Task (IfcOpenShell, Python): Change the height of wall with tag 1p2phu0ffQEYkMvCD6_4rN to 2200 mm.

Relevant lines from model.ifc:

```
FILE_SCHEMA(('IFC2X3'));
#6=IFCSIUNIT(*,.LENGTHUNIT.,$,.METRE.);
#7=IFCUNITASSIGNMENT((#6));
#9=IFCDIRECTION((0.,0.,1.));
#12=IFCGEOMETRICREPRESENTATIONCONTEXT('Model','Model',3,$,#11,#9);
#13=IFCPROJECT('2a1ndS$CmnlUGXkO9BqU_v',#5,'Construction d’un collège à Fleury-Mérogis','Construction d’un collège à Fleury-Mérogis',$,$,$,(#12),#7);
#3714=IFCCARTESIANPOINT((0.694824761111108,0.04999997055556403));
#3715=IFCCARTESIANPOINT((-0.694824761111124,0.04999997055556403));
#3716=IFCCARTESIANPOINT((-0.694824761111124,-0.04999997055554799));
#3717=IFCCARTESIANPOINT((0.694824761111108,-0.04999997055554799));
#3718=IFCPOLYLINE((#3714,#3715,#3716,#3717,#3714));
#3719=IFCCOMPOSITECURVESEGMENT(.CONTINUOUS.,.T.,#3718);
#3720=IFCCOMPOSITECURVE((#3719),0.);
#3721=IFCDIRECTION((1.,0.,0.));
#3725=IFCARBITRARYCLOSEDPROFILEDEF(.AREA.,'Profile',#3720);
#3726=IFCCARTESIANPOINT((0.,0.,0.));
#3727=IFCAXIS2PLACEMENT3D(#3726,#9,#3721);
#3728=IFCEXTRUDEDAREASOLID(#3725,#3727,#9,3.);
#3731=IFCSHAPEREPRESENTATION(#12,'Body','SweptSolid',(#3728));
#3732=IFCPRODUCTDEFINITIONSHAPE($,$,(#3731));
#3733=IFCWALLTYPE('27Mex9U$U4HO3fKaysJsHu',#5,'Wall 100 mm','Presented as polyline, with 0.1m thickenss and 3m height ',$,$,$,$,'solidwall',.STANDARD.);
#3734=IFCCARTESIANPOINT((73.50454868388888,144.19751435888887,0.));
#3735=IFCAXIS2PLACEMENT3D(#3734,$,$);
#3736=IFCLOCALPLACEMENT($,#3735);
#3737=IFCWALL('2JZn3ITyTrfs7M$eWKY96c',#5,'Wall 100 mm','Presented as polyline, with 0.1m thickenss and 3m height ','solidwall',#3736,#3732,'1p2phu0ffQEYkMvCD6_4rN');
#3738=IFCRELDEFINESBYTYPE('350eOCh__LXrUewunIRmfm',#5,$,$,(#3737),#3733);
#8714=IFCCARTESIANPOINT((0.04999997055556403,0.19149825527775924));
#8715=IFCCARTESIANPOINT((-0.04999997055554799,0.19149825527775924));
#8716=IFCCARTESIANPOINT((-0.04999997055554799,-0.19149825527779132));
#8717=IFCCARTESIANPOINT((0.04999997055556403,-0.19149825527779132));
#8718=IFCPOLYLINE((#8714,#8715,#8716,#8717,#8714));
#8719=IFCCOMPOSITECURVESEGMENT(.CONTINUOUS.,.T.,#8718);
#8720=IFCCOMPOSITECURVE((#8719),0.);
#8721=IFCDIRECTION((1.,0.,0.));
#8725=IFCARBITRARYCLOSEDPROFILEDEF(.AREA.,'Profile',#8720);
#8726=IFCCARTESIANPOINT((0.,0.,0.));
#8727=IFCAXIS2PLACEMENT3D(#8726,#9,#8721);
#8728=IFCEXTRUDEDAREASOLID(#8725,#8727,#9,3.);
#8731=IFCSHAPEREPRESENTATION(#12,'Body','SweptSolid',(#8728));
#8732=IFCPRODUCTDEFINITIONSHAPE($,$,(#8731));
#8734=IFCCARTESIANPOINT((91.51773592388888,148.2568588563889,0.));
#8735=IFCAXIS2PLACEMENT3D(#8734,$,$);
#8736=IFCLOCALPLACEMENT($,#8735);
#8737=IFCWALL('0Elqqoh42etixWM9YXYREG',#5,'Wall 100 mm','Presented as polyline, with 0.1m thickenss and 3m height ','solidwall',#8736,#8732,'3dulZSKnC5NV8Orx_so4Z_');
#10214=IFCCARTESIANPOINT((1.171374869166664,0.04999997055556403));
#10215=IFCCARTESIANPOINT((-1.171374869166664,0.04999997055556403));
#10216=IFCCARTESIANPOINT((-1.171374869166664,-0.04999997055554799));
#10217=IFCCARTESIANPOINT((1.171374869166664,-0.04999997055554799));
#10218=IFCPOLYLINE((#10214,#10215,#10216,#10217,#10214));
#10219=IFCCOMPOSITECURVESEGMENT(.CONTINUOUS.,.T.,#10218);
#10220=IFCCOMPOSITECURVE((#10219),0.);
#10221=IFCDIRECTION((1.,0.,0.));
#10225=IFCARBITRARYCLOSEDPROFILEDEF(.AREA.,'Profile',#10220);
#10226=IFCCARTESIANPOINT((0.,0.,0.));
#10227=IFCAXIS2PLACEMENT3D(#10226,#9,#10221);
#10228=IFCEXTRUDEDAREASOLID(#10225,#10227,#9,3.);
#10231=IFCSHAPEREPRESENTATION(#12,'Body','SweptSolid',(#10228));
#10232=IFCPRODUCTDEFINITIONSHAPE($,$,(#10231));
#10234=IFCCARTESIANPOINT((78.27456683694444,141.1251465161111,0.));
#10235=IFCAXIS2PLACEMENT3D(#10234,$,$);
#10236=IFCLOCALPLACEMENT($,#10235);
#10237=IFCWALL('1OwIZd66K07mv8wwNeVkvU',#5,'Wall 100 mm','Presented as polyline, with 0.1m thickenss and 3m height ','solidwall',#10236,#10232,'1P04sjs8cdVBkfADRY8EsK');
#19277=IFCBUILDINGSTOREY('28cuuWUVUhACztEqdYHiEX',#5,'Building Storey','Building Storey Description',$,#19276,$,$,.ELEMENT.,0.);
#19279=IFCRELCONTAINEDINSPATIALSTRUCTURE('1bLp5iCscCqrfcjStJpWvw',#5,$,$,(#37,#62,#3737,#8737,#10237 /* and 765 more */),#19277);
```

```python
import ifcopenshell
import ifcopenshell.geom
import ifcopenshell.util.shape

model = ifcopenshell.open("model.ifc")
settings = ifcopenshell.geom.settings()


def volume(element):
    """Net volume in cubic metres, openings subtracted."""
    shape = ifcopenshell.geom.create_shape(settings, element)
    return ifcopenshell.util.shape.get_volume(shape.geometry)


wall = model.by_id(3737)
before = volume(wall)

body = next(r for r in wall.Representation.Representations if r.RepresentationIdentifier == "Body")
solid = body.Items[0]
old_height = solid.Depth
solid.Depth = 2.2
after = volume(wall)

print(f"height {old_height:g} -> {solid.Depth:g}, volume {before:.3f} -> {after:.3f} m3")

model.write("model_updated.ifc")
```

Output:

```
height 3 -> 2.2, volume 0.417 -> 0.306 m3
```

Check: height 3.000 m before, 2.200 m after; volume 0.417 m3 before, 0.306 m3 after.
